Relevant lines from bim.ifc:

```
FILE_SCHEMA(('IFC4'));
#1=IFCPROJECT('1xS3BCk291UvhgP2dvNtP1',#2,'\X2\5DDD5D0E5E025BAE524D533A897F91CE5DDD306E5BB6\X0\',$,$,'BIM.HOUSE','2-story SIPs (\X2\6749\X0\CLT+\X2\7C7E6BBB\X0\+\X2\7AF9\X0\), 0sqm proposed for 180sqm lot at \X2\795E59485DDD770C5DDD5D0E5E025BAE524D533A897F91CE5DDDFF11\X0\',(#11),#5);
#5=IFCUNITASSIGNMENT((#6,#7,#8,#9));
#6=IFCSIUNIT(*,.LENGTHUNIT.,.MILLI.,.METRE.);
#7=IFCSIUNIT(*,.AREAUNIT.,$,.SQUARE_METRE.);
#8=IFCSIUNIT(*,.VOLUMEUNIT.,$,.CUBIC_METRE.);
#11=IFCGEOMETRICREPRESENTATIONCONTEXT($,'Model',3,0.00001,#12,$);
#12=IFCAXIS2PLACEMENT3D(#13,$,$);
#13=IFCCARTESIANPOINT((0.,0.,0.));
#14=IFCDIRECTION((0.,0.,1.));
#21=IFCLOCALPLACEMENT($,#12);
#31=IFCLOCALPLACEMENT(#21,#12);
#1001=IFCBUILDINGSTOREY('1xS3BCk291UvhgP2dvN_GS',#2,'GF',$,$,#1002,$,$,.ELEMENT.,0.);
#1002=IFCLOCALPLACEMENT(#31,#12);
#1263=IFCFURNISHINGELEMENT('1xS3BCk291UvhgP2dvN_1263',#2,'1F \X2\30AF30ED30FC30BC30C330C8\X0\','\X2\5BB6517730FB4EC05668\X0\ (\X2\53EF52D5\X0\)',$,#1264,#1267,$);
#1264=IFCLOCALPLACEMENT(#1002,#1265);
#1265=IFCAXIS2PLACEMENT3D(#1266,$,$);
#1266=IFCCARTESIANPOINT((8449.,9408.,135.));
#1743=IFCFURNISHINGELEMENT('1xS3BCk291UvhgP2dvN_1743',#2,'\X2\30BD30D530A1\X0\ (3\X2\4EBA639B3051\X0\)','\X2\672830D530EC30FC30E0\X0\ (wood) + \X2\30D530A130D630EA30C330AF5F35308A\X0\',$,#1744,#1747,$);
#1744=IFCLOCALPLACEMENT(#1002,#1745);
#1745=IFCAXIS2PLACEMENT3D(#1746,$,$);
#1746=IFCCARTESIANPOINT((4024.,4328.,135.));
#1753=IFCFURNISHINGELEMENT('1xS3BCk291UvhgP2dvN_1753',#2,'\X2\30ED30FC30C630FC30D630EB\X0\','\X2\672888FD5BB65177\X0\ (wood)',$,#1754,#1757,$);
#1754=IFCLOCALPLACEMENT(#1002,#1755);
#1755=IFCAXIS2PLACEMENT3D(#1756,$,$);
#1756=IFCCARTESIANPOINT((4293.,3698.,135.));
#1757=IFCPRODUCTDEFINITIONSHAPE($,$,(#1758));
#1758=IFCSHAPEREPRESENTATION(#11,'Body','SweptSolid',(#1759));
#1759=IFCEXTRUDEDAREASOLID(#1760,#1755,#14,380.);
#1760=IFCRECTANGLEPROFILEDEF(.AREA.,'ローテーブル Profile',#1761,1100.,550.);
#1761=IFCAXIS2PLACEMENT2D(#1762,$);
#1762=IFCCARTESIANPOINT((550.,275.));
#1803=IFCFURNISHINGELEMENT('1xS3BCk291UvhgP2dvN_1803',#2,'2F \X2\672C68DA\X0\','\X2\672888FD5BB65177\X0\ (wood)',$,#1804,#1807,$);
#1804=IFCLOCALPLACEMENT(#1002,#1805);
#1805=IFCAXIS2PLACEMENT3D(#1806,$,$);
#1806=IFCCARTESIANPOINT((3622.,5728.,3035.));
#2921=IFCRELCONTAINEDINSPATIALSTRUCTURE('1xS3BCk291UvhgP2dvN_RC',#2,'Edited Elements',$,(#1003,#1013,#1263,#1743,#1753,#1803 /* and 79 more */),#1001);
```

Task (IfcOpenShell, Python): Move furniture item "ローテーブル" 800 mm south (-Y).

```python
import ifcopenshell
import ifcopenshell.api.geometry
import ifcopenshell.util.placement

model = ifcopenshell.open("bim.ifc")

item = model.by_id(1753)
matrix = ifcopenshell.util.placement.get_local_placement(item.ObjectPlacement)
matrix[1, 3] -= 800.0
ifcopenshell.api.geometry.edit_object_placement(model, product=item, matrix=matrix, is_si=False)

print(ifcopenshell.util.placement.get_local_placement(item.ObjectPlacement).round(3) + 0.0)

model.write("bim-out.ifc")
```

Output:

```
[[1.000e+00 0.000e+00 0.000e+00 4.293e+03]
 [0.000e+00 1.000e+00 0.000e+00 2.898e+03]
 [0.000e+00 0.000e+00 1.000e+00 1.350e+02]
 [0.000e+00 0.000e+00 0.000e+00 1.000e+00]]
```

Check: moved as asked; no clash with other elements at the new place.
